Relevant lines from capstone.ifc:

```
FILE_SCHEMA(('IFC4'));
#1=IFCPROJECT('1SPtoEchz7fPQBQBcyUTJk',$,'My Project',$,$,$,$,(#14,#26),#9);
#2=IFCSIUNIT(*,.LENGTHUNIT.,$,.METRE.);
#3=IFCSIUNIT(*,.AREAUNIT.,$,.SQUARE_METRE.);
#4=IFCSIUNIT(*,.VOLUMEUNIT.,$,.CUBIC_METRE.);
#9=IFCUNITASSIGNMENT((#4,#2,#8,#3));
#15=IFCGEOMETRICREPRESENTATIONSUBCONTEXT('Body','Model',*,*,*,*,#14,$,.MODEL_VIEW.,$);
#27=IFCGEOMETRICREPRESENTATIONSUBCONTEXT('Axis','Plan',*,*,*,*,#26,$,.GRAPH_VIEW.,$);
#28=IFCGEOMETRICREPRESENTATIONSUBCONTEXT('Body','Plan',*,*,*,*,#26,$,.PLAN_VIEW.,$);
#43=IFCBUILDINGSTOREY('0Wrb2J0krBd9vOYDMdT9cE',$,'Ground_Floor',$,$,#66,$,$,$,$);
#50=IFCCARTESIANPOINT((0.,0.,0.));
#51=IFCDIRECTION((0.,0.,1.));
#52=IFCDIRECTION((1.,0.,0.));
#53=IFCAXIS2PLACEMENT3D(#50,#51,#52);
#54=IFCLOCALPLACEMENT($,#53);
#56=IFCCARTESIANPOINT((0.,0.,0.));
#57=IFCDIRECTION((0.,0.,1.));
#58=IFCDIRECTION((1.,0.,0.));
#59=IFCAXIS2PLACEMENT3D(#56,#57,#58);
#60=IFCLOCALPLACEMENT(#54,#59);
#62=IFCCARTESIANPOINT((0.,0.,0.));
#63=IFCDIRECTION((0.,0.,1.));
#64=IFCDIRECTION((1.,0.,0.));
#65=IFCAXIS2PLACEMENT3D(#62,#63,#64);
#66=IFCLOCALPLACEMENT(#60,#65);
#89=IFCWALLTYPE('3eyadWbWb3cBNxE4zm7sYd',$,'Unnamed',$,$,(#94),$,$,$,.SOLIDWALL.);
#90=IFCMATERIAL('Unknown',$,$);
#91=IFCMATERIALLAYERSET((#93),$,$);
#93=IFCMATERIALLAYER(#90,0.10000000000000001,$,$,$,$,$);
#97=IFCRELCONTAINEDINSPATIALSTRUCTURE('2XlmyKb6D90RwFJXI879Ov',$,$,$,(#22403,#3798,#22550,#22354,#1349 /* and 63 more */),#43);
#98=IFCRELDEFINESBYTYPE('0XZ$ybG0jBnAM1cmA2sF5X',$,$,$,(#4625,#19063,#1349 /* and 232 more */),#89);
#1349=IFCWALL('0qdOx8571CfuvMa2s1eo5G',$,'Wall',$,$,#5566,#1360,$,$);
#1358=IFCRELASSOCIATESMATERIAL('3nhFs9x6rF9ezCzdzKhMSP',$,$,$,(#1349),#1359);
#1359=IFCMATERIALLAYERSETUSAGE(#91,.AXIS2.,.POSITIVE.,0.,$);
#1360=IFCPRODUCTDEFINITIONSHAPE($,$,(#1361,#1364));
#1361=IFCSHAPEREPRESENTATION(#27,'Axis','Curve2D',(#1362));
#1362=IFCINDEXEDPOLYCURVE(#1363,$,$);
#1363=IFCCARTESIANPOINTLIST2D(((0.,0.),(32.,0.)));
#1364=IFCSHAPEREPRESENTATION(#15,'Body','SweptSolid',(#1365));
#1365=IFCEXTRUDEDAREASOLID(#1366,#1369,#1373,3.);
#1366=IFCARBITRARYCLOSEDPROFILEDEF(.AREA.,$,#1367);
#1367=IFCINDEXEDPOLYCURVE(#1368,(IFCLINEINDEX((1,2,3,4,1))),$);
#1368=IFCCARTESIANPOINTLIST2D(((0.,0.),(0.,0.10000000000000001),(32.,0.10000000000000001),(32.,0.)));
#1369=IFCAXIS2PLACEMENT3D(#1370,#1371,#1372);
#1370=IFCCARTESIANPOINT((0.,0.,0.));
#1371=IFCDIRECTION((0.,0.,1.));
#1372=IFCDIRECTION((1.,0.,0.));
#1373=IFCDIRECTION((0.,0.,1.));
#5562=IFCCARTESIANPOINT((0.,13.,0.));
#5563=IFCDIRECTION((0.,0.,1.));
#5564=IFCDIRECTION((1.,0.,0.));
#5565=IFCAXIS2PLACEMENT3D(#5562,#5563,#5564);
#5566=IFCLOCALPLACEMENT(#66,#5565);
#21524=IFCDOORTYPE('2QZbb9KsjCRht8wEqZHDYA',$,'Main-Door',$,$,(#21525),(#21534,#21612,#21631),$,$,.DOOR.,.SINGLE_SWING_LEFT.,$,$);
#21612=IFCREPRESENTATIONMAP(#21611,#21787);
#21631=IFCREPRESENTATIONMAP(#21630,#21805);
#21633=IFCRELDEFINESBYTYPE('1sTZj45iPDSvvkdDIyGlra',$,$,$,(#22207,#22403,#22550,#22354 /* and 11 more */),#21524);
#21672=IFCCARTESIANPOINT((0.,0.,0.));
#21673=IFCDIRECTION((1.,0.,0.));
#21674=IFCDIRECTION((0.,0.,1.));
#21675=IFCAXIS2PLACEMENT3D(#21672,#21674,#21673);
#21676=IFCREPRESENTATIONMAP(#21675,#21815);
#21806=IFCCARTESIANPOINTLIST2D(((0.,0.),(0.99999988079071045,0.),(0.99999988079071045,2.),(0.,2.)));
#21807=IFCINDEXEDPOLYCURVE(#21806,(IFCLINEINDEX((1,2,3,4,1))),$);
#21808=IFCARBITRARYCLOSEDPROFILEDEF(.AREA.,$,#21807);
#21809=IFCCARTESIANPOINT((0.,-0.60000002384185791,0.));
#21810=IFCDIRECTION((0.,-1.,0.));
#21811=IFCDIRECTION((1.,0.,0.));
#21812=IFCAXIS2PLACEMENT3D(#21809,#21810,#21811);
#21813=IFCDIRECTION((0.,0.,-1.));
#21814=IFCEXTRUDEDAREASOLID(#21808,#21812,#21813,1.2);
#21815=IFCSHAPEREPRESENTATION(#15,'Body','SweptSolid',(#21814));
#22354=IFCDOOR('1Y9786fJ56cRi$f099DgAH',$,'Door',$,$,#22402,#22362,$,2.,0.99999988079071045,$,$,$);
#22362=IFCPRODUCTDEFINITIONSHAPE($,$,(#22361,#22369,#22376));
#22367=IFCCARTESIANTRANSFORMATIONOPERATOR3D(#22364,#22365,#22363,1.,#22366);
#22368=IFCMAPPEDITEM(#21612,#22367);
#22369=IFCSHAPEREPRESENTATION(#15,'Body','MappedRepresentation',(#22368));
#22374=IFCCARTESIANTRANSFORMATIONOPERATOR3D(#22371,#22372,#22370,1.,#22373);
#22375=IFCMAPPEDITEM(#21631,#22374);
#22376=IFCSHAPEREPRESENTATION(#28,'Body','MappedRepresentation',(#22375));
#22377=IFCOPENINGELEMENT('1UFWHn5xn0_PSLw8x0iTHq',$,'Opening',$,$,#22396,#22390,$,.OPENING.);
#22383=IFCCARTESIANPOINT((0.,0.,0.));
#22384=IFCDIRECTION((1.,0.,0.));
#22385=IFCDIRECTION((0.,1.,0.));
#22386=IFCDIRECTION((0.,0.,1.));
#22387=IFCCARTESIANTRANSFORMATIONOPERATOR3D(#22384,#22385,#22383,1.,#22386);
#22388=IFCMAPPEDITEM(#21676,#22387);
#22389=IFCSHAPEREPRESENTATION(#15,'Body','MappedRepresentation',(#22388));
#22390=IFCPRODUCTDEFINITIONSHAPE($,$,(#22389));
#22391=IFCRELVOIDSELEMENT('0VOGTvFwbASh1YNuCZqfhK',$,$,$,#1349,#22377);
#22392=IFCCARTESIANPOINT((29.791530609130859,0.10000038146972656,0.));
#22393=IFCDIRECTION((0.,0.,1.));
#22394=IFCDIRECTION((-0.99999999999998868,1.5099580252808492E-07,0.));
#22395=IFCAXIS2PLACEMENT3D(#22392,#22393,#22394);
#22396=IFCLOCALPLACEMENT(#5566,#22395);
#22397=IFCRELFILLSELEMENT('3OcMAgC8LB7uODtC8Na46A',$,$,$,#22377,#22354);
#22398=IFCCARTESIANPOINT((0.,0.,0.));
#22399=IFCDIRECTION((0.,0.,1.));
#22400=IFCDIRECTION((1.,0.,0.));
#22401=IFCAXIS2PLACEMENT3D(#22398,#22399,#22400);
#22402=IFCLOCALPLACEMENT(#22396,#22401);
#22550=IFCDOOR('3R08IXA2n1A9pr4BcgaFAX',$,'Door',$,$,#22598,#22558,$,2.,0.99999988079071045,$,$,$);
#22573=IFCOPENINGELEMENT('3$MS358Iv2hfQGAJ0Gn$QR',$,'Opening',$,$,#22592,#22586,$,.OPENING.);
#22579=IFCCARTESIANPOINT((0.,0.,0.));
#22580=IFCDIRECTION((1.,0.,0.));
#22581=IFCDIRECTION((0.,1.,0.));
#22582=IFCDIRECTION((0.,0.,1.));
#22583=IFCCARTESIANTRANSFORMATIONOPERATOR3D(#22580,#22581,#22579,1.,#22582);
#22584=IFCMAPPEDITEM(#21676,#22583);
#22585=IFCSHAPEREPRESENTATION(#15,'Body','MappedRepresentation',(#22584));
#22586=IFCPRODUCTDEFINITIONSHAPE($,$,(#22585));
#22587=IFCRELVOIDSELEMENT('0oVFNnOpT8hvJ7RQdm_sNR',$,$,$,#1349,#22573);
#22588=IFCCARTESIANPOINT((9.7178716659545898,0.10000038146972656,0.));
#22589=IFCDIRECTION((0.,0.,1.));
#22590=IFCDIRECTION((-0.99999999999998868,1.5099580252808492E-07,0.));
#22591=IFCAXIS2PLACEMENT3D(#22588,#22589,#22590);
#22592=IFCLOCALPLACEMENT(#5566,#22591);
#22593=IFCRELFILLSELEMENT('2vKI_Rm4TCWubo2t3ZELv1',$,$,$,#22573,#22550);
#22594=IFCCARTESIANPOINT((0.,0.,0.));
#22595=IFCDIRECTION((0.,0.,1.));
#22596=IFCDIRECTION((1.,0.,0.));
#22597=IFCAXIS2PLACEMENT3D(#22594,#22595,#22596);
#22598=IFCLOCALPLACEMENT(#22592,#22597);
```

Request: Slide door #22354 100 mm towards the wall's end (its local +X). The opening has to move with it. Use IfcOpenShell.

```python
import ifcopenshell
import ifcopenshell.api.geometry
import ifcopenshell.util.placement
import ifcopenshell.util.unit

model = ifcopenshell.open("capstone.ifc")
unit_scale = ifcopenshell.util.unit.calculate_unit_scale(model)

door = model.by_guid("1Y9786fJ56cRi$f099DgAH")
opening = door.FillsVoids[0].RelatingOpeningElement
wall = opening.VoidsElements[0].RelatingBuildingElement

wall_matrix = ifcopenshell.util.placement.get_local_placement(wall.ObjectPlacement)
shift = wall_matrix[:3, 0] * 0.1 / unit_scale
before = ifcopenshell.util.placement.get_local_placement(door.ObjectPlacement)[:3, 3].copy()

# The door is placed relative to its opening, so it follows when the opening moves.
matrix = ifcopenshell.util.placement.get_local_placement(opening.ObjectPlacement)
matrix[:3, 3] += shift
ifcopenshell.api.geometry.edit_object_placement(
    model, product=opening, matrix=matrix, is_si=False, should_transform_children=True
)

after = ifcopenshell.util.placement.get_local_placement(door.ObjectPlacement)[:3, 3]
print("door moved by", (after - before).round(3) + 0.0)

model.write("capstone_edited.ifc")
```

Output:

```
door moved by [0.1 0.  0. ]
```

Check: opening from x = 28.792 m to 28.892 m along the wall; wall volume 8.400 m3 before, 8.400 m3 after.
